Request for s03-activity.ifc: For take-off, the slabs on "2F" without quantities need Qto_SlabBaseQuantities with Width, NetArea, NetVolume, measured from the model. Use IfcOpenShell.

First a look at what the model holds.

```python
import ifcopenshell
import ifcopenshell.util.element
import ifcopenshell.util.unit

model = ifcopenshell.open("s03-activity.ifc")
print(model.schema)
for unit_type in ("LENGTHUNIT", "AREAUNIT", "VOLUMEUNIT"):
    print(unit_type, ifcopenshell.util.unit.calculate_unit_scale(model, unit_type))
storey = next(s for s in model.by_type("IfcBuildingStorey") if s.Name == "2F")
slabs = [e for e in ifcopenshell.util.element.get_decomposition(storey) if e.is_a("IfcSlab")]
for e in sorted(slabs, key=lambda e: e.id()):
    print(e.id(), e.is_a(), e.Name, list(ifcopenshell.util.element.get_psets(e, qtos_only=True)), sep=" | ")
```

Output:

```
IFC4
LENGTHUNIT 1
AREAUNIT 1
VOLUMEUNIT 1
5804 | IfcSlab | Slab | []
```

```python
import ifcopenshell
import ifcopenshell.api.pset
import ifcopenshell.geom
import ifcopenshell.util.element
import ifcopenshell.util.shape
import ifcopenshell.util.unit

model = ifcopenshell.open("s03-activity.ifc")
unit_scale = ifcopenshell.util.unit.calculate_unit_scale(model)
area_scale = ifcopenshell.util.unit.calculate_unit_scale(model, "AREAUNIT")
volume_scale = ifcopenshell.util.unit.calculate_unit_scale(model, "VOLUMEUNIT")
settings = ifcopenshell.geom.settings()

storey = next(s for s in model.by_type("IfcBuildingStorey") if s.Name == "2F")
slabs = [e for e in ifcopenshell.util.element.get_decomposition(storey) if e.is_a("IfcSlab")]

for e in sorted(slabs, key=lambda e: e.id()):
    if ifcopenshell.util.element.get_psets(e, qtos_only=True, should_inherit=False):
        continue
    # Geometry comes back in metres, in the element's own axes.
    shape = ifcopenshell.geom.create_shape(settings, e)
    values = {
        "Width": ifcopenshell.util.shape.get_z(shape.geometry) / unit_scale,
        "NetArea": ifcopenshell.util.shape.get_footprint_area(shape.geometry) / area_scale,
        "NetVolume": ifcopenshell.util.shape.get_volume(shape.geometry) / volume_scale,
    }
    qto = ifcopenshell.api.pset.add_qto(model, product=e, name="Qto_SlabBaseQuantities")
    ifcopenshell.api.pset.edit_qto(model, qto=qto, properties=values)
    print(e.id(), {k: round(v, 3) for k, v in values.items()})

model.write("s03-activity-out.ifc")
```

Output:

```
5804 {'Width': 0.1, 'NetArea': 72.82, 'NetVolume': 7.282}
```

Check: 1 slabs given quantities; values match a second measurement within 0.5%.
